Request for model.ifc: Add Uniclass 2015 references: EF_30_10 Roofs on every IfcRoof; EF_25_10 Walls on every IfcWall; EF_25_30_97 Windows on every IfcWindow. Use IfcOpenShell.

First a look at what the model holds.

```python
import ifcopenshell

model = ifcopenshell.open("model.ifc")
print(model.schema)
print("classifications:", [c.Name for c in model.by_type("IfcClassification")])
for ifc_class in ("IfcDoor", "IfcRoof", "IfcStair", "IfcWall", "IfcWindow"):
    print(ifc_class, len(model.by_type(ifc_class)))
```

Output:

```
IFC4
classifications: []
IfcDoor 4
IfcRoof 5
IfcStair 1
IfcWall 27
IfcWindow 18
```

```python
import ifcopenshell
import ifcopenshell.api.classification

model = ifcopenshell.open("model.ifc")

system = ifcopenshell.api.classification.add_classification(model, classification="Uniclass 2015")

codes = {
    "IfcRoof": ("EF_30_10", "Roofs"),
    "IfcWall": ("EF_25_10", "Walls"),
    "IfcWindow": ("EF_25_30_97", "Windows"),
}
for ifc_class, (code, name) in codes.items():
    products = model.by_type(ifc_class)
    ifcopenshell.api.classification.add_reference(
        model, products=products, classification=system, identification=code, name=name
    )
    print(code, len(products))

model.write("model_v2.ifc")
```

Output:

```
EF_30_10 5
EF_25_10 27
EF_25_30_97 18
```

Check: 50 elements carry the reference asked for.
